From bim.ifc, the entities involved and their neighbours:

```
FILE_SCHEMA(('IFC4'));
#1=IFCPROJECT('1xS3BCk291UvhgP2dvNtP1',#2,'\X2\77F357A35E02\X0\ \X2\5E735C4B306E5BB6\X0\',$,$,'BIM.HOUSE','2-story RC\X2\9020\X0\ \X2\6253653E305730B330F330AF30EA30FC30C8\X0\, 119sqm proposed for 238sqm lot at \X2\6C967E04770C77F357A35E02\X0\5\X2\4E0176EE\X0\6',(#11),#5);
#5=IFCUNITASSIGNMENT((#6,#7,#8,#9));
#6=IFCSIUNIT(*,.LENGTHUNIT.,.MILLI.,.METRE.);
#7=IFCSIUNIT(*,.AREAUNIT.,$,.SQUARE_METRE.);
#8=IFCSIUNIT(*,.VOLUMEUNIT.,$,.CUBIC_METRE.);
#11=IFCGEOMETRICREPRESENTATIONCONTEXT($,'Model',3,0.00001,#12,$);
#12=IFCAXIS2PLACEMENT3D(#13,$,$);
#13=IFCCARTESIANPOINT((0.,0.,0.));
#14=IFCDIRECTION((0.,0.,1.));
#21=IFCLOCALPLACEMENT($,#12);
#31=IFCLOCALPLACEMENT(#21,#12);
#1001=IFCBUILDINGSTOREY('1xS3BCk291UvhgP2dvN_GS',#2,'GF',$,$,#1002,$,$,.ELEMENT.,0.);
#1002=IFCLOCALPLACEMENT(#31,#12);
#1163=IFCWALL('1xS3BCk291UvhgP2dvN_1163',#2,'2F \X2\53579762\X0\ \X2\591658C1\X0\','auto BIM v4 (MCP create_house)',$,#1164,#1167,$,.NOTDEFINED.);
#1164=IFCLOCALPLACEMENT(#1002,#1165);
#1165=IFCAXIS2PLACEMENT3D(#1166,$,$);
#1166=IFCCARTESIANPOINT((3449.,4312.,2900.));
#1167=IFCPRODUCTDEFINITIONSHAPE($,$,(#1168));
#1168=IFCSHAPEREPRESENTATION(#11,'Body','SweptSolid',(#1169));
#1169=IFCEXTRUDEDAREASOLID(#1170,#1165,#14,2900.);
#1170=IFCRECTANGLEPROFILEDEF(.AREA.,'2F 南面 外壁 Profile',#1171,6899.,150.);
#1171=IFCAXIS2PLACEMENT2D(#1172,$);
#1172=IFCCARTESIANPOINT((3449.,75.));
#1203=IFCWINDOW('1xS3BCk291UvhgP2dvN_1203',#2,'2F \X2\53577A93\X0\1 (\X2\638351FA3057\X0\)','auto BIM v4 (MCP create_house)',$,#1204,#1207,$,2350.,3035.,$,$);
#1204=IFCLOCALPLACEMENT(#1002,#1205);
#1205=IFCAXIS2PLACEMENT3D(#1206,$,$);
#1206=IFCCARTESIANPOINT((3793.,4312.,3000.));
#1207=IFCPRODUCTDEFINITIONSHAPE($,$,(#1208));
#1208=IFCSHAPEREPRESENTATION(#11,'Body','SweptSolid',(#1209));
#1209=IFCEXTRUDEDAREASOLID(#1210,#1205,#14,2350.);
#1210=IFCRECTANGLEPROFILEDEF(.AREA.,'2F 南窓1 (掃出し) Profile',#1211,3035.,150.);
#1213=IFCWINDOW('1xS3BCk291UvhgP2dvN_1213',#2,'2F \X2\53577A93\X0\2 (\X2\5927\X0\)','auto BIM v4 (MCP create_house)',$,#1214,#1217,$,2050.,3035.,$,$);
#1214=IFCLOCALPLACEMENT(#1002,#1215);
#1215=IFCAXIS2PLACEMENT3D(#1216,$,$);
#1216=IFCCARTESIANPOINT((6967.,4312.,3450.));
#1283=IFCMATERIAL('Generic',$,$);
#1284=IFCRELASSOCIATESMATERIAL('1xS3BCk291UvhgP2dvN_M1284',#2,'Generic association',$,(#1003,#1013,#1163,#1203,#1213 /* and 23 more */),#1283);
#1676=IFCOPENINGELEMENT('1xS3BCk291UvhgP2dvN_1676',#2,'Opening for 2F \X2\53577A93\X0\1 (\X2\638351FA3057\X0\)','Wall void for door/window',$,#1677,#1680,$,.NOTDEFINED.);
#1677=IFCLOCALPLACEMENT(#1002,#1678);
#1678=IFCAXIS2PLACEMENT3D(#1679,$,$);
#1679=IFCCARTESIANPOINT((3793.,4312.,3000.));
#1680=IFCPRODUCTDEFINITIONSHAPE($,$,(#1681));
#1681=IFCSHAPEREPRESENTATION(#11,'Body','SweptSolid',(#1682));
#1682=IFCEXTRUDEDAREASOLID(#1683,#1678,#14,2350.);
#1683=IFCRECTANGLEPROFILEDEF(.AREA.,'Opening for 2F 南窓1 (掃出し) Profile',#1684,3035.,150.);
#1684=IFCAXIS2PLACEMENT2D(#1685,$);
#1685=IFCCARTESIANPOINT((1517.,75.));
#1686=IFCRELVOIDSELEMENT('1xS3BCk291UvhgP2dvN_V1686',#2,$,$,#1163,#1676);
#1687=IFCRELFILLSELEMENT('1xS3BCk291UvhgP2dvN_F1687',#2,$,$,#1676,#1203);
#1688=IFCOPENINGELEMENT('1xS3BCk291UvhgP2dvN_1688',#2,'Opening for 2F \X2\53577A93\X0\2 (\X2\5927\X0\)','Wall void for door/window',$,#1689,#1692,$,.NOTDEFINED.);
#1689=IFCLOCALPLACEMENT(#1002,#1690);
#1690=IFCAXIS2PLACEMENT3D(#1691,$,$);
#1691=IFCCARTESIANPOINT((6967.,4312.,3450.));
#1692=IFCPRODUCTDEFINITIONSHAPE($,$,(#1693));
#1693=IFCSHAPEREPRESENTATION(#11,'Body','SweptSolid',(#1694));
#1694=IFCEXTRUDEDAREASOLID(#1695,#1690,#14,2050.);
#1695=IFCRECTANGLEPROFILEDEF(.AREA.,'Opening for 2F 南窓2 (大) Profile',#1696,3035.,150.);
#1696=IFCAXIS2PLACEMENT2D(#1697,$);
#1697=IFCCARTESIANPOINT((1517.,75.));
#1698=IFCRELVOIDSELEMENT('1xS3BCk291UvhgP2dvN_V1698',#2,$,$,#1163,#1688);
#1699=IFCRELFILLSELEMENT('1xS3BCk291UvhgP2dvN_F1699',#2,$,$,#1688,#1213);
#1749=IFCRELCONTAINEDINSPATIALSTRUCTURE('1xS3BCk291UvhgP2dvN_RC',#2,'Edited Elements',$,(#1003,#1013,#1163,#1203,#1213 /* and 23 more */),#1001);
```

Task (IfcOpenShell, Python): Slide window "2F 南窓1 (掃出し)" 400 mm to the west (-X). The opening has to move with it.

```python
import ifcopenshell
import ifcopenshell.api.geometry
import ifcopenshell.util.placement

model = ifcopenshell.open("bim.ifc")

window = model.by_guid("1xS3BCk291UvhgP2dvN_1203")
opening = window.FillsVoids[0].RelatingOpeningElement
wall = opening.VoidsElements[0].RelatingBuildingElement

wall_matrix = ifcopenshell.util.placement.get_local_placement(wall.ObjectPlacement)
shift = wall_matrix[:3, 0] * -400.0
before = ifcopenshell.util.placement.get_local_placement(window.ObjectPlacement)[:3, 3].copy()

# The window is not placed relative to its opening, so move both.
for product in (opening, window):
    matrix = ifcopenshell.util.placement.get_local_placement(product.ObjectPlacement)
    matrix[:3, 3] += shift
    ifcopenshell.api.geometry.edit_object_placement(model, product=product, matrix=matrix, is_si=False)

after = ifcopenshell.util.placement.get_local_placement(window.ObjectPlacement)[:3, 3]
print("window moved by", (after - before).round(3) + 0.0)

model.write("bim_rev.ifc")
```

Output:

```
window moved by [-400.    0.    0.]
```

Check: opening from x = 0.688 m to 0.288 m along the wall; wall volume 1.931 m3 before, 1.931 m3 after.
